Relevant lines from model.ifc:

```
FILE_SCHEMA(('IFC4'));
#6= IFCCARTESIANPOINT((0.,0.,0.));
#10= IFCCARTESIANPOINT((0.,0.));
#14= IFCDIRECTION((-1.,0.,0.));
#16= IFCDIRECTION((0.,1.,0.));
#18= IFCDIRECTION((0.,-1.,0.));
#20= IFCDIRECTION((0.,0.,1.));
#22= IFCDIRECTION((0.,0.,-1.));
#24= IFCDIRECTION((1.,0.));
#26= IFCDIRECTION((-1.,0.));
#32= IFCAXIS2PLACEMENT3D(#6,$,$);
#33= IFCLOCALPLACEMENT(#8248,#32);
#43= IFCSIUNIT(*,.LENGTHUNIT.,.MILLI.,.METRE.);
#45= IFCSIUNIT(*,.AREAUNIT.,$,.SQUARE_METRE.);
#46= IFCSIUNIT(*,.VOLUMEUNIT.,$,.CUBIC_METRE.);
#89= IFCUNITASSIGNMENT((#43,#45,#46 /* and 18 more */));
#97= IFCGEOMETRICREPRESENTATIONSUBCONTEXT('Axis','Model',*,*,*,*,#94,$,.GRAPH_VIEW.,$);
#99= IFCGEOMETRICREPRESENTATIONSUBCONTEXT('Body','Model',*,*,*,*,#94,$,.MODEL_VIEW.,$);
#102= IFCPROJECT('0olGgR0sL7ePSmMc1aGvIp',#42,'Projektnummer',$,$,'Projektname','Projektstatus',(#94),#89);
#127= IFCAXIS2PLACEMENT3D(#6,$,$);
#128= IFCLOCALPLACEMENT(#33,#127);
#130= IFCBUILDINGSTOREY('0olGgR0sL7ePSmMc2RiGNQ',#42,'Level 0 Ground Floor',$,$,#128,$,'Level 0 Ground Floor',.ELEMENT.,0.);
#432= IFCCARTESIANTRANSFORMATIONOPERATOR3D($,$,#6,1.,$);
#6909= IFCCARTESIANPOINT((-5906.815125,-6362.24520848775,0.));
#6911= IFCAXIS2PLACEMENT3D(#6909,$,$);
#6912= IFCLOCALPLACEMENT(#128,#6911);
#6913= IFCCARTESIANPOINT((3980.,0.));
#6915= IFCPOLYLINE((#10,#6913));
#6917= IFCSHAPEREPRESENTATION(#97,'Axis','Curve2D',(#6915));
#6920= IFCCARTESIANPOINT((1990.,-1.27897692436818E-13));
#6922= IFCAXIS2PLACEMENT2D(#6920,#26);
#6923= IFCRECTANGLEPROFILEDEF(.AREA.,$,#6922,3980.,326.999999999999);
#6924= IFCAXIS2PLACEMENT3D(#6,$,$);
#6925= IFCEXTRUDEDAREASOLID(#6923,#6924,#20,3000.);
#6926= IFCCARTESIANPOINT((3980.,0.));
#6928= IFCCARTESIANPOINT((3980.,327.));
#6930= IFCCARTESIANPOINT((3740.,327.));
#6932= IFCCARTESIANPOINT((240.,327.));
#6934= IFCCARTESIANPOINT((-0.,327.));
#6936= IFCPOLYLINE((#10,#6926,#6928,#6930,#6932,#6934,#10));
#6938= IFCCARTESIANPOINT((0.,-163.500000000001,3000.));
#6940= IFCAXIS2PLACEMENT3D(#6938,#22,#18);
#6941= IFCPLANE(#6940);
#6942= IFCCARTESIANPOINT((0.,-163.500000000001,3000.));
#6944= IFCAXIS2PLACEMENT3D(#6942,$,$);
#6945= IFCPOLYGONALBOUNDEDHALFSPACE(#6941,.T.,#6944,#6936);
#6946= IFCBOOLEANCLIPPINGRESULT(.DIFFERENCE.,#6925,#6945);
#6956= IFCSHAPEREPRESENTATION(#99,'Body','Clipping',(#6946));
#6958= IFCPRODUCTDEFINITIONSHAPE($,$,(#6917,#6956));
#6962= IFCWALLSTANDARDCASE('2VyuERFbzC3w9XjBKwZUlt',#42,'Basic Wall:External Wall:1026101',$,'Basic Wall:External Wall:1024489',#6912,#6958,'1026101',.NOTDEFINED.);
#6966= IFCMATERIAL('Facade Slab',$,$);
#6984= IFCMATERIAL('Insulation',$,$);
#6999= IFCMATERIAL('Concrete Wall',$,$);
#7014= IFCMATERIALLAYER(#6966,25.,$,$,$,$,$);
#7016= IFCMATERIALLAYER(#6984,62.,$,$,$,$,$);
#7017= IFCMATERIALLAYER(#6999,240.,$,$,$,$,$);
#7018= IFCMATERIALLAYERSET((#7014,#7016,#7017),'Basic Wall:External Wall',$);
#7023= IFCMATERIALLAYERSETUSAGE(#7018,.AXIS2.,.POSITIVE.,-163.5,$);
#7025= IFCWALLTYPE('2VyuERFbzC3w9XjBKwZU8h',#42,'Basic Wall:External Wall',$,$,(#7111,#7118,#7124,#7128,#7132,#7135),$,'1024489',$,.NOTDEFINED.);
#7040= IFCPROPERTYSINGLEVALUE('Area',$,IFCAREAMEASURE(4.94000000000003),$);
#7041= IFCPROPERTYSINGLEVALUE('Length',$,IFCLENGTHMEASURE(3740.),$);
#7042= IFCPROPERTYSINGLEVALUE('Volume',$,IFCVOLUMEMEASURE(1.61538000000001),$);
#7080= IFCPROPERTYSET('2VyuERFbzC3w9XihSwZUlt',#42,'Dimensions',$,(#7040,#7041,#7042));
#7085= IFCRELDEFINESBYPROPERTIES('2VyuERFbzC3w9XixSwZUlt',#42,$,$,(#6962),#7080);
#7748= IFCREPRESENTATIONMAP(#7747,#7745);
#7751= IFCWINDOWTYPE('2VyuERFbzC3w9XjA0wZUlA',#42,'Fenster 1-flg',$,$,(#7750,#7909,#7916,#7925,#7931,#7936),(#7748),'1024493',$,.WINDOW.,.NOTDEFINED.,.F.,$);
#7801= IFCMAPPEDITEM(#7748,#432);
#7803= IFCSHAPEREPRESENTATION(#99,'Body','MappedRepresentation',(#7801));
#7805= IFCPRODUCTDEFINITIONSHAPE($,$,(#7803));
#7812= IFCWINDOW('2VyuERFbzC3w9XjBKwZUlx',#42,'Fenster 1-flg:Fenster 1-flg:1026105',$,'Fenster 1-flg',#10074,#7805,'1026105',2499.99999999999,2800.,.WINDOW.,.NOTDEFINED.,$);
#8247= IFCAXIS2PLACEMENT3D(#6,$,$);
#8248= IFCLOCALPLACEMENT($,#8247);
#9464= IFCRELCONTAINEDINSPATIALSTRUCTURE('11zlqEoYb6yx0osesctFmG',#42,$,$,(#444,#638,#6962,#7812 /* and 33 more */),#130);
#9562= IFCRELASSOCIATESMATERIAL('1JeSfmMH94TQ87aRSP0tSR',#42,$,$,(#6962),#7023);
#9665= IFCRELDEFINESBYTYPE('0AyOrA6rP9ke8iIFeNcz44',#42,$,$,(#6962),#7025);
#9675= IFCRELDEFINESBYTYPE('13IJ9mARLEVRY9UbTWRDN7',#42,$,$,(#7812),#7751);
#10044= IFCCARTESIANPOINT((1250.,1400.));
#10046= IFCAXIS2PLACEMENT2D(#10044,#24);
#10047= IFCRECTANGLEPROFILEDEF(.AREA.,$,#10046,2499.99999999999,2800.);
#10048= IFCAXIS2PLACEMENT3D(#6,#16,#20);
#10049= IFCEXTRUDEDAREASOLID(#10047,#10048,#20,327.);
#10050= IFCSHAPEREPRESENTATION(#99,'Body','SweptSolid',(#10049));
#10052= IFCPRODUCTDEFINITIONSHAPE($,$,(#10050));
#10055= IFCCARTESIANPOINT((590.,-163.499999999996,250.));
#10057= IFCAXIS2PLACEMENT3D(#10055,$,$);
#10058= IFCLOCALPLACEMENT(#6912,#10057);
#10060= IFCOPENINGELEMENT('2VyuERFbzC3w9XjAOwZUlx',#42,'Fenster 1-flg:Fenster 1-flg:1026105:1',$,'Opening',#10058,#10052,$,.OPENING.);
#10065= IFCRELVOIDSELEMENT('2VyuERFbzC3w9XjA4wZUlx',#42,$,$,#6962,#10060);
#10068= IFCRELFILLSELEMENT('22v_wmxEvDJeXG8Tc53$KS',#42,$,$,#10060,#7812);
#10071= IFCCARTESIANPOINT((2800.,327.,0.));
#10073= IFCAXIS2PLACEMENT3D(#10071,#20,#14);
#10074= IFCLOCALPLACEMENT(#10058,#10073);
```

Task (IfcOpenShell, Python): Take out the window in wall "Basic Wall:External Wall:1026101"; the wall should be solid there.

```python
import ifcopenshell
import ifcopenshell.api.feature
import ifcopenshell.api.pset
import ifcopenshell.api.root
import ifcopenshell.geom
import ifcopenshell.util.element
import ifcopenshell.util.shape
import ifcopenshell.util.unit

model = ifcopenshell.open("model.ifc")
area_scale = ifcopenshell.util.unit.calculate_unit_scale(model, "AREAUNIT")
volume_scale = ifcopenshell.util.unit.calculate_unit_scale(model, "VOLUMEUNIT")
settings = ifcopenshell.geom.settings()


def volume(element):
    """Net volume in cubic metres, openings subtracted."""
    shape = ifcopenshell.geom.create_shape(settings, element)
    return ifcopenshell.util.shape.get_volume(shape.geometry)


window = model.by_guid("2VyuERFbzC3w9XjBKwZUlx")
opening = window.FillsVoids[0].RelatingOpeningElement
wall = opening.VoidsElements[0].RelatingBuildingElement
before = volume(wall)

ifcopenshell.api.root.remove_product(model, product=window)
ifcopenshell.api.feature.remove_feature(model, feature=opening)

after = volume(wall)
thickness = 0.327  # wall thickness in metres

# Update the wall's stored quantities.
pset = model.by_id(ifcopenshell.util.element.get_pset(wall, "Dimensions", should_inherit=False)["id"])
ifcopenshell.api.pset.edit_pset(model, pset=pset, properties={
    "Area": model.create_entity("IfcAreaMeasure", after / thickness / area_scale),
    "Volume": model.create_entity("IfcVolumeMeasure", after / volume_scale),
})

print(f"wall volume {before:.3f} -> {after:.3f} m3")

model.write("model_v2.ifc")
```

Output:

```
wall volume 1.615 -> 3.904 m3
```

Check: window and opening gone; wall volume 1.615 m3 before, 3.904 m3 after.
